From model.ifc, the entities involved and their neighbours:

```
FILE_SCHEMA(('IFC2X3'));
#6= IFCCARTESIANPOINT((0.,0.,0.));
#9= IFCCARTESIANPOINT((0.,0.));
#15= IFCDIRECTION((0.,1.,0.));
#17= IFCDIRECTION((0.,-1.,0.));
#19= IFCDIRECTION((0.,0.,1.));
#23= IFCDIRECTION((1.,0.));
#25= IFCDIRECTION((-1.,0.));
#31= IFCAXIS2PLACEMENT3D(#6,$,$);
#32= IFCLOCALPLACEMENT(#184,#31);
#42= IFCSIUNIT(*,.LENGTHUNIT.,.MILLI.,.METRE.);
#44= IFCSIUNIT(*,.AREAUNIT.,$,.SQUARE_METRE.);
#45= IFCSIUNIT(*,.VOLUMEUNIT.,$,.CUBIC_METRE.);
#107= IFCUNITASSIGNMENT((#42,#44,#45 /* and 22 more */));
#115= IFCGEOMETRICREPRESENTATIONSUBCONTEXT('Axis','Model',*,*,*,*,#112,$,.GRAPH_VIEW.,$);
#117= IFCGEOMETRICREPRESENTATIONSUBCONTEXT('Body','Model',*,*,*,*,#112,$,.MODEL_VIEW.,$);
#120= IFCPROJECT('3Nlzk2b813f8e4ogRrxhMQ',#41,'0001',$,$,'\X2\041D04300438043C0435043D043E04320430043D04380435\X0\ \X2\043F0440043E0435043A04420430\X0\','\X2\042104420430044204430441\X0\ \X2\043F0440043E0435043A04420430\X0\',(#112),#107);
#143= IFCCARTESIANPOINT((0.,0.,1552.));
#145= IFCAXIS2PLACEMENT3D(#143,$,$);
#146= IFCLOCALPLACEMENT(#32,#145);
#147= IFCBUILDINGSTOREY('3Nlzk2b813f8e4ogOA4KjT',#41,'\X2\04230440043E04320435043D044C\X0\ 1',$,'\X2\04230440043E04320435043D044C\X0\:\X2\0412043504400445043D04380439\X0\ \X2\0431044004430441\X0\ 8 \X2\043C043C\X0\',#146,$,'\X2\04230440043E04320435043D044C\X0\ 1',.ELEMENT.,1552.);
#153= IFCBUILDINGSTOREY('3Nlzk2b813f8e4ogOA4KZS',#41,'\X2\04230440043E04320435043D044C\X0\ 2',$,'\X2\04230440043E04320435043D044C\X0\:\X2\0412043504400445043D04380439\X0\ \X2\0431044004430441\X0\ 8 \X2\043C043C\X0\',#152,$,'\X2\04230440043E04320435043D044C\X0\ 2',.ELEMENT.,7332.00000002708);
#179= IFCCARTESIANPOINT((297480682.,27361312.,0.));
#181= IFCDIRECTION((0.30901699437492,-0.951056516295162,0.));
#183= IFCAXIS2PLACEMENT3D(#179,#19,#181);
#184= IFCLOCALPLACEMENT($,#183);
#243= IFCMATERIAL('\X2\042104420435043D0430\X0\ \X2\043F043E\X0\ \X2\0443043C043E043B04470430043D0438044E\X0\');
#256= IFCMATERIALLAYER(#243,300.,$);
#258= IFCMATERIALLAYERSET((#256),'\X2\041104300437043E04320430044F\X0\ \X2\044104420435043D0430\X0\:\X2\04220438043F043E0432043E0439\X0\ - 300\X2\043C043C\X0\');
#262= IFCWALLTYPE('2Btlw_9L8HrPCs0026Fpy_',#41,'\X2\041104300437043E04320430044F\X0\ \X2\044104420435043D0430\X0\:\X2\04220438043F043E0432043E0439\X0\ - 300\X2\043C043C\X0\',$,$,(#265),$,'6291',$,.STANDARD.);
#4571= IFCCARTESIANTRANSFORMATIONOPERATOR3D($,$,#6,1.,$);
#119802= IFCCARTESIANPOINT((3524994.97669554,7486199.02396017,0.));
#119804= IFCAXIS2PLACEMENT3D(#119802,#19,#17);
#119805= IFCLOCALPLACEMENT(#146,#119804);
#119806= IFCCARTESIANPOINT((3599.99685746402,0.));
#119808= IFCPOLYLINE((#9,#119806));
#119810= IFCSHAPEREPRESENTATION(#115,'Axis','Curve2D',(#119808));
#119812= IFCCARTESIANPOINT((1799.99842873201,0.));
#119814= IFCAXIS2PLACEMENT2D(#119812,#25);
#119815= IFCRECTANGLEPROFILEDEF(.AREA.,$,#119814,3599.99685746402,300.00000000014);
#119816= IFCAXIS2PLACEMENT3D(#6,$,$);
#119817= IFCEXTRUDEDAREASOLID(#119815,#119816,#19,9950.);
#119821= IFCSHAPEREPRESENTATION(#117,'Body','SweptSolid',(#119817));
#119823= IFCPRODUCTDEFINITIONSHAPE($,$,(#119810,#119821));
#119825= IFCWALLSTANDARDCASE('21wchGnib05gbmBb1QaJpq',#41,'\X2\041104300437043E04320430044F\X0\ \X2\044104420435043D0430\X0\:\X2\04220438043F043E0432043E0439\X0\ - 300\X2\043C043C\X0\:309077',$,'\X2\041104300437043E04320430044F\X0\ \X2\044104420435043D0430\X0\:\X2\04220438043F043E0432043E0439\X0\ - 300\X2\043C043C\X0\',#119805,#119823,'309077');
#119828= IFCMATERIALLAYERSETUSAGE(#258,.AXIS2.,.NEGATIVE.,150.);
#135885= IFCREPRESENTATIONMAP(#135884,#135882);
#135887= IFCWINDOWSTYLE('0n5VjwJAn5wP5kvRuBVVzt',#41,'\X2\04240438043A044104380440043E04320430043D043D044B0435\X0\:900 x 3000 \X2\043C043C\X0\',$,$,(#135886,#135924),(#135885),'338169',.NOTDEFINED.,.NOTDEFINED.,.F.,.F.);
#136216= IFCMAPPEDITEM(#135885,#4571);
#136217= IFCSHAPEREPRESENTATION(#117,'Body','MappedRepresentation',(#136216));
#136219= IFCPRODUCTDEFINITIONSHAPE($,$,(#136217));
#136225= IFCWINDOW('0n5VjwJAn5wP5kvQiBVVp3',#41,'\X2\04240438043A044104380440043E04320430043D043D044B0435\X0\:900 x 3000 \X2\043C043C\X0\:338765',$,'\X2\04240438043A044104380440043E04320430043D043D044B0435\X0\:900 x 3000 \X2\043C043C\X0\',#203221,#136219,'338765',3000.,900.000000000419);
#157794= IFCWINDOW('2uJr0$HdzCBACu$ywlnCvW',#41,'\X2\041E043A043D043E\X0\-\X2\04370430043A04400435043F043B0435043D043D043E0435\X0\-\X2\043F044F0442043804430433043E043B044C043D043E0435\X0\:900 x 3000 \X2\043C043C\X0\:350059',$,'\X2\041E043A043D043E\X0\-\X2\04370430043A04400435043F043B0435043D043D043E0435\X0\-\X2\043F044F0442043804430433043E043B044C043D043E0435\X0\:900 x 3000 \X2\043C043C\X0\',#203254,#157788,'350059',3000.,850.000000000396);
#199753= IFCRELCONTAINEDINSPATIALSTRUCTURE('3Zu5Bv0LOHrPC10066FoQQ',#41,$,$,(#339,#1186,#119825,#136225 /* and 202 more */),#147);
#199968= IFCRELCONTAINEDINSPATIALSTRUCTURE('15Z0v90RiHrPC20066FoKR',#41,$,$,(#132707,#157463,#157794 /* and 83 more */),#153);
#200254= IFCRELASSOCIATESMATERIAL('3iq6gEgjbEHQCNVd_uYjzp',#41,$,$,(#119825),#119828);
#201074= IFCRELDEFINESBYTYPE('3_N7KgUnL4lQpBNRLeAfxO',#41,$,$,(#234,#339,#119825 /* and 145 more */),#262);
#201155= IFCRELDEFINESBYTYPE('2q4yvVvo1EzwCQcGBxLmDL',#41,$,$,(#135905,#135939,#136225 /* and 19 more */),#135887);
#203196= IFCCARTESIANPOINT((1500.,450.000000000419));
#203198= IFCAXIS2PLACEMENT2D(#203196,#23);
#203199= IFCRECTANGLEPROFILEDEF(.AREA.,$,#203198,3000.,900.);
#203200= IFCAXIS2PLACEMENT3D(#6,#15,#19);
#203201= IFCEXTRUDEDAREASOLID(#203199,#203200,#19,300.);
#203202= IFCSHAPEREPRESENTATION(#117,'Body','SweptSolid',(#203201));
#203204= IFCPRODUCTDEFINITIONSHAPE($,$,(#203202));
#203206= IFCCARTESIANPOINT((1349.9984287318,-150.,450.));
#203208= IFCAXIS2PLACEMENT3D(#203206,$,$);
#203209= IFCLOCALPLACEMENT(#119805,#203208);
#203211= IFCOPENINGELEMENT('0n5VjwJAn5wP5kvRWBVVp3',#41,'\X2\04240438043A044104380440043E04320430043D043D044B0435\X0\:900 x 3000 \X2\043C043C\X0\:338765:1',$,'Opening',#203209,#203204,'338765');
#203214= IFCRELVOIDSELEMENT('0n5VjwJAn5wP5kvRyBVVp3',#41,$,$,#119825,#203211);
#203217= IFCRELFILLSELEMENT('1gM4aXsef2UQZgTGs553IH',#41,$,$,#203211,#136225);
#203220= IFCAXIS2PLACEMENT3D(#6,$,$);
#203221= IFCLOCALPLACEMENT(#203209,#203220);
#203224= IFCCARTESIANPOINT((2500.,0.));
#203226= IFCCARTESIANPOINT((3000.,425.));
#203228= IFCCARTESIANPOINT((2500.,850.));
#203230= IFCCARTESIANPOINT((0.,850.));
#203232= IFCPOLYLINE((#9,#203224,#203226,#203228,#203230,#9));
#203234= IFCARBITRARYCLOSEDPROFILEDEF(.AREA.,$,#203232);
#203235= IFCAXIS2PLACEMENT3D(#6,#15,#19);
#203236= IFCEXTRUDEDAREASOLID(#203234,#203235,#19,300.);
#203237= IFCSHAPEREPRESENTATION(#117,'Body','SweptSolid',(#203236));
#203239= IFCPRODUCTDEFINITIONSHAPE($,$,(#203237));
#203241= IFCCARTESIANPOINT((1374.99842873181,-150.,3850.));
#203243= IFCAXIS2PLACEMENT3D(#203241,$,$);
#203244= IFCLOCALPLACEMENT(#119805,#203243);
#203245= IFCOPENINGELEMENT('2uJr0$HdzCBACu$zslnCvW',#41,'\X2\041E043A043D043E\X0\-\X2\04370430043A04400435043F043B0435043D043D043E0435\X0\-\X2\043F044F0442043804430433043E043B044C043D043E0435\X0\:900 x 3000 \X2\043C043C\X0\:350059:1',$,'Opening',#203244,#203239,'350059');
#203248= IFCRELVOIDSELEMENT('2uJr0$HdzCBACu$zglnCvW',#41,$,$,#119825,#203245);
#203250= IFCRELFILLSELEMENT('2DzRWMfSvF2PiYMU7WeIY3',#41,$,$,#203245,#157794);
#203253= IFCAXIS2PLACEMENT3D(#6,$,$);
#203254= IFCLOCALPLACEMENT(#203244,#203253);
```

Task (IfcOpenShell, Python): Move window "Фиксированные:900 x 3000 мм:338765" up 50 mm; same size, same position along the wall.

```python
import numpy as np
import ifcopenshell
import ifcopenshell.api.geometry
import ifcopenshell.util.placement
import ifcopenshell.util.unit

model = ifcopenshell.open("model.ifc")
unit_scale = ifcopenshell.util.unit.calculate_unit_scale(model)

window = model.by_guid("0n5VjwJAn5wP5kvQiBVVp3")
opening = window.FillsVoids[0].RelatingOpeningElement
dz = 50.0

shift = np.array([0.0, 0.0, dz])
# The window is placed relative to its opening, so it follows when the opening moves.
matrix = ifcopenshell.util.placement.get_local_placement(opening.ObjectPlacement)
matrix[:3, 3] += shift
ifcopenshell.api.geometry.edit_object_placement(
    model, product=opening, matrix=matrix, is_si=False, should_transform_children=True
)

print(f"moved by {dz * unit_scale:+.3f} m")

model.write("model-out.ifc")
```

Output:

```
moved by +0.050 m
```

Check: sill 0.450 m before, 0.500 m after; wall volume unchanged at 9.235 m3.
